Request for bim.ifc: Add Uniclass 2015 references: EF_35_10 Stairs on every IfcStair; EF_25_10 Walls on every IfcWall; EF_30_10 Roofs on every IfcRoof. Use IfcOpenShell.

First a look at what the model holds.

```python
import ifcopenshell

model = ifcopenshell.open("bim.ifc")
print(model.schema)
print("classifications:", [c.Name for c in model.by_type("IfcClassification")])
for ifc_class in ("IfcDoor", "IfcRoof", "IfcStair", "IfcWall", "IfcWindow"):
    print(ifc_class, len(model.by_type(ifc_class)))
```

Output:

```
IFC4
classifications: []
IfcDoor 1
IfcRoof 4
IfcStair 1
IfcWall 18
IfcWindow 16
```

```python
import ifcopenshell
import ifcopenshell.api.classification

model = ifcopenshell.open("bim.ifc")

system = ifcopenshell.api.classification.add_classification(model, classification="Uniclass 2015")

codes = {
    "IfcStair": ("EF_35_10", "Stairs"),
    "IfcWall": ("EF_25_10", "Walls"),
    "IfcRoof": ("EF_30_10", "Roofs"),
}
for ifc_class, (code, name) in codes.items():
    products = model.by_type(ifc_class)
    ifcopenshell.api.classification.add_reference(
        model, products=products, classification=system, identification=code, name=name
    )
    print(code, len(products))

model.write("bim_rev.ifc")
```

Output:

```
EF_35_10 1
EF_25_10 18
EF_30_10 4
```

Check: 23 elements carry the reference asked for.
